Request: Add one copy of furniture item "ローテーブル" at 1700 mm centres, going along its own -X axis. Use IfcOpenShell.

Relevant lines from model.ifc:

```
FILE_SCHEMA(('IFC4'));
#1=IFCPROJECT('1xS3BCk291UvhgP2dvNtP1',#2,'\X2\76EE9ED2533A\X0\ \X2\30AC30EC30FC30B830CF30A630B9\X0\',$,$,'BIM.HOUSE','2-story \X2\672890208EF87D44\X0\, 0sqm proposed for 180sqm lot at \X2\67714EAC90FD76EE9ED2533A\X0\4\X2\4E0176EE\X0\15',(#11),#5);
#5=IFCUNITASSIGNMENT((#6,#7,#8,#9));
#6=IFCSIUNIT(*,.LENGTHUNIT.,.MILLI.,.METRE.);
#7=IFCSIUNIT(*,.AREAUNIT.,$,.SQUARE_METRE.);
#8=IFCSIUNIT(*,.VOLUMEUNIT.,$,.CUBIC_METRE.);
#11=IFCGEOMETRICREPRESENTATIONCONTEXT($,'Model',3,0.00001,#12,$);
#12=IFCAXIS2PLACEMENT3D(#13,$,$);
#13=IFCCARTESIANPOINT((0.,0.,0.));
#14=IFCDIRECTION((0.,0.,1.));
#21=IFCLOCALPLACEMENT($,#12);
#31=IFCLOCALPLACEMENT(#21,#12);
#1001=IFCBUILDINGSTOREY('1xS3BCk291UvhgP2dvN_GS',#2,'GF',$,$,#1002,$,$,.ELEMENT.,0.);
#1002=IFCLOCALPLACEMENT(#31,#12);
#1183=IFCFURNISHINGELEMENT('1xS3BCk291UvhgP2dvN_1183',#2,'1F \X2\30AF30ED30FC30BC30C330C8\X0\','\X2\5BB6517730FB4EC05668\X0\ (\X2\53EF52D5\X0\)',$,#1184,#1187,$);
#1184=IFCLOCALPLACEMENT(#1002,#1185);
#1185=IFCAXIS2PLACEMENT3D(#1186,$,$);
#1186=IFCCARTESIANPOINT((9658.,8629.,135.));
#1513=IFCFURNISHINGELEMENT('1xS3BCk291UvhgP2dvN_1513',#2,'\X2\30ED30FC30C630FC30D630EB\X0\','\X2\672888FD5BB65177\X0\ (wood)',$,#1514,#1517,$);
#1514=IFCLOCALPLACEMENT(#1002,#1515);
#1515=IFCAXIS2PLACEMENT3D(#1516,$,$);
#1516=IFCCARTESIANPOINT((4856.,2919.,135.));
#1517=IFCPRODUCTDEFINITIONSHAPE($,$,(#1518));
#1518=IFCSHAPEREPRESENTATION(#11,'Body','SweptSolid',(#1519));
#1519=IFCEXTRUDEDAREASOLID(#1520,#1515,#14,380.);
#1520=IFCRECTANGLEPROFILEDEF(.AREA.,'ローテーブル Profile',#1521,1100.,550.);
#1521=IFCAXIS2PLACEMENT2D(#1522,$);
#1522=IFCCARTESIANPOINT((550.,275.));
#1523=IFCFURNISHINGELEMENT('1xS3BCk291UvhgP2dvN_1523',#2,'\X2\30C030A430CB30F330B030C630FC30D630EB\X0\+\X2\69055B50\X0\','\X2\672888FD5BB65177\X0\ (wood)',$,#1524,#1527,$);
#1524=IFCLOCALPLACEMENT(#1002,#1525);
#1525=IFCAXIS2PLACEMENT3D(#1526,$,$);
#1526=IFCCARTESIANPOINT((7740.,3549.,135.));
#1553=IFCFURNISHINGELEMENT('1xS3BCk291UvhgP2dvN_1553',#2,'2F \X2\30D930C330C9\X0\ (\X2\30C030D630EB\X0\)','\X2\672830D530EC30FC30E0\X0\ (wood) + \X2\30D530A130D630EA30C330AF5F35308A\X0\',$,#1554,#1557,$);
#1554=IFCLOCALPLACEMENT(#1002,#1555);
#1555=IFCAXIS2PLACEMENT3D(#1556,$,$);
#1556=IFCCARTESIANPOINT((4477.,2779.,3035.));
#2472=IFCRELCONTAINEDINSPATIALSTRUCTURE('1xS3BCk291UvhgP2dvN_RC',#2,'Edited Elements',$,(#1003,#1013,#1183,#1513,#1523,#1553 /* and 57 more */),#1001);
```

```python
import ifcopenshell
import ifcopenshell.api.geometry
import ifcopenshell.api.root
import ifcopenshell.util.element
import ifcopenshell.util.placement
import ifcopenshell.util.unit

model = ifcopenshell.open("model.ifc")
unit_scale = ifcopenshell.util.unit.calculate_unit_scale(model)


def reuse_history(source, copy):
    """copy_class also copies each property set's owner history, people and application; keep the originals."""
    for rel in copy.IsDefinedBy:
        if rel.is_a("IfcRelDefinesByProperties") and (history := rel.RelatingPropertyDefinition.OwnerHistory):
            rel.RelatingPropertyDefinition.OwnerHistory = source.OwnerHistory
            ifcopenshell.util.element.remove_deep2(model, history)


source = model.by_id(1513)
base = ifcopenshell.util.placement.get_local_placement(source.ObjectPlacement)
step = -base[:3, 0] * 1.7 / unit_scale

for i in range(1, 2):
    copy = ifcopenshell.api.root.copy_class(model, product=source)
    copy.Representation = ifcopenshell.util.element.copy_deep(
        model, source.Representation, exclude=["IfcGeometricRepresentationContext", "IfcRepresentationMap"]
    )
    reuse_history(source, copy)
    matrix = base.copy()
    matrix[:3, 3] += i * step
    print("added at", matrix[:3, 3].round(3) + 0.0)
    ifcopenshell.api.geometry.edit_object_placement(model, product=copy, matrix=matrix, is_si=False)

model.write("model_v2.ifc")
```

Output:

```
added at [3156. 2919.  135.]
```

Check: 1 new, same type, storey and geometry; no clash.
